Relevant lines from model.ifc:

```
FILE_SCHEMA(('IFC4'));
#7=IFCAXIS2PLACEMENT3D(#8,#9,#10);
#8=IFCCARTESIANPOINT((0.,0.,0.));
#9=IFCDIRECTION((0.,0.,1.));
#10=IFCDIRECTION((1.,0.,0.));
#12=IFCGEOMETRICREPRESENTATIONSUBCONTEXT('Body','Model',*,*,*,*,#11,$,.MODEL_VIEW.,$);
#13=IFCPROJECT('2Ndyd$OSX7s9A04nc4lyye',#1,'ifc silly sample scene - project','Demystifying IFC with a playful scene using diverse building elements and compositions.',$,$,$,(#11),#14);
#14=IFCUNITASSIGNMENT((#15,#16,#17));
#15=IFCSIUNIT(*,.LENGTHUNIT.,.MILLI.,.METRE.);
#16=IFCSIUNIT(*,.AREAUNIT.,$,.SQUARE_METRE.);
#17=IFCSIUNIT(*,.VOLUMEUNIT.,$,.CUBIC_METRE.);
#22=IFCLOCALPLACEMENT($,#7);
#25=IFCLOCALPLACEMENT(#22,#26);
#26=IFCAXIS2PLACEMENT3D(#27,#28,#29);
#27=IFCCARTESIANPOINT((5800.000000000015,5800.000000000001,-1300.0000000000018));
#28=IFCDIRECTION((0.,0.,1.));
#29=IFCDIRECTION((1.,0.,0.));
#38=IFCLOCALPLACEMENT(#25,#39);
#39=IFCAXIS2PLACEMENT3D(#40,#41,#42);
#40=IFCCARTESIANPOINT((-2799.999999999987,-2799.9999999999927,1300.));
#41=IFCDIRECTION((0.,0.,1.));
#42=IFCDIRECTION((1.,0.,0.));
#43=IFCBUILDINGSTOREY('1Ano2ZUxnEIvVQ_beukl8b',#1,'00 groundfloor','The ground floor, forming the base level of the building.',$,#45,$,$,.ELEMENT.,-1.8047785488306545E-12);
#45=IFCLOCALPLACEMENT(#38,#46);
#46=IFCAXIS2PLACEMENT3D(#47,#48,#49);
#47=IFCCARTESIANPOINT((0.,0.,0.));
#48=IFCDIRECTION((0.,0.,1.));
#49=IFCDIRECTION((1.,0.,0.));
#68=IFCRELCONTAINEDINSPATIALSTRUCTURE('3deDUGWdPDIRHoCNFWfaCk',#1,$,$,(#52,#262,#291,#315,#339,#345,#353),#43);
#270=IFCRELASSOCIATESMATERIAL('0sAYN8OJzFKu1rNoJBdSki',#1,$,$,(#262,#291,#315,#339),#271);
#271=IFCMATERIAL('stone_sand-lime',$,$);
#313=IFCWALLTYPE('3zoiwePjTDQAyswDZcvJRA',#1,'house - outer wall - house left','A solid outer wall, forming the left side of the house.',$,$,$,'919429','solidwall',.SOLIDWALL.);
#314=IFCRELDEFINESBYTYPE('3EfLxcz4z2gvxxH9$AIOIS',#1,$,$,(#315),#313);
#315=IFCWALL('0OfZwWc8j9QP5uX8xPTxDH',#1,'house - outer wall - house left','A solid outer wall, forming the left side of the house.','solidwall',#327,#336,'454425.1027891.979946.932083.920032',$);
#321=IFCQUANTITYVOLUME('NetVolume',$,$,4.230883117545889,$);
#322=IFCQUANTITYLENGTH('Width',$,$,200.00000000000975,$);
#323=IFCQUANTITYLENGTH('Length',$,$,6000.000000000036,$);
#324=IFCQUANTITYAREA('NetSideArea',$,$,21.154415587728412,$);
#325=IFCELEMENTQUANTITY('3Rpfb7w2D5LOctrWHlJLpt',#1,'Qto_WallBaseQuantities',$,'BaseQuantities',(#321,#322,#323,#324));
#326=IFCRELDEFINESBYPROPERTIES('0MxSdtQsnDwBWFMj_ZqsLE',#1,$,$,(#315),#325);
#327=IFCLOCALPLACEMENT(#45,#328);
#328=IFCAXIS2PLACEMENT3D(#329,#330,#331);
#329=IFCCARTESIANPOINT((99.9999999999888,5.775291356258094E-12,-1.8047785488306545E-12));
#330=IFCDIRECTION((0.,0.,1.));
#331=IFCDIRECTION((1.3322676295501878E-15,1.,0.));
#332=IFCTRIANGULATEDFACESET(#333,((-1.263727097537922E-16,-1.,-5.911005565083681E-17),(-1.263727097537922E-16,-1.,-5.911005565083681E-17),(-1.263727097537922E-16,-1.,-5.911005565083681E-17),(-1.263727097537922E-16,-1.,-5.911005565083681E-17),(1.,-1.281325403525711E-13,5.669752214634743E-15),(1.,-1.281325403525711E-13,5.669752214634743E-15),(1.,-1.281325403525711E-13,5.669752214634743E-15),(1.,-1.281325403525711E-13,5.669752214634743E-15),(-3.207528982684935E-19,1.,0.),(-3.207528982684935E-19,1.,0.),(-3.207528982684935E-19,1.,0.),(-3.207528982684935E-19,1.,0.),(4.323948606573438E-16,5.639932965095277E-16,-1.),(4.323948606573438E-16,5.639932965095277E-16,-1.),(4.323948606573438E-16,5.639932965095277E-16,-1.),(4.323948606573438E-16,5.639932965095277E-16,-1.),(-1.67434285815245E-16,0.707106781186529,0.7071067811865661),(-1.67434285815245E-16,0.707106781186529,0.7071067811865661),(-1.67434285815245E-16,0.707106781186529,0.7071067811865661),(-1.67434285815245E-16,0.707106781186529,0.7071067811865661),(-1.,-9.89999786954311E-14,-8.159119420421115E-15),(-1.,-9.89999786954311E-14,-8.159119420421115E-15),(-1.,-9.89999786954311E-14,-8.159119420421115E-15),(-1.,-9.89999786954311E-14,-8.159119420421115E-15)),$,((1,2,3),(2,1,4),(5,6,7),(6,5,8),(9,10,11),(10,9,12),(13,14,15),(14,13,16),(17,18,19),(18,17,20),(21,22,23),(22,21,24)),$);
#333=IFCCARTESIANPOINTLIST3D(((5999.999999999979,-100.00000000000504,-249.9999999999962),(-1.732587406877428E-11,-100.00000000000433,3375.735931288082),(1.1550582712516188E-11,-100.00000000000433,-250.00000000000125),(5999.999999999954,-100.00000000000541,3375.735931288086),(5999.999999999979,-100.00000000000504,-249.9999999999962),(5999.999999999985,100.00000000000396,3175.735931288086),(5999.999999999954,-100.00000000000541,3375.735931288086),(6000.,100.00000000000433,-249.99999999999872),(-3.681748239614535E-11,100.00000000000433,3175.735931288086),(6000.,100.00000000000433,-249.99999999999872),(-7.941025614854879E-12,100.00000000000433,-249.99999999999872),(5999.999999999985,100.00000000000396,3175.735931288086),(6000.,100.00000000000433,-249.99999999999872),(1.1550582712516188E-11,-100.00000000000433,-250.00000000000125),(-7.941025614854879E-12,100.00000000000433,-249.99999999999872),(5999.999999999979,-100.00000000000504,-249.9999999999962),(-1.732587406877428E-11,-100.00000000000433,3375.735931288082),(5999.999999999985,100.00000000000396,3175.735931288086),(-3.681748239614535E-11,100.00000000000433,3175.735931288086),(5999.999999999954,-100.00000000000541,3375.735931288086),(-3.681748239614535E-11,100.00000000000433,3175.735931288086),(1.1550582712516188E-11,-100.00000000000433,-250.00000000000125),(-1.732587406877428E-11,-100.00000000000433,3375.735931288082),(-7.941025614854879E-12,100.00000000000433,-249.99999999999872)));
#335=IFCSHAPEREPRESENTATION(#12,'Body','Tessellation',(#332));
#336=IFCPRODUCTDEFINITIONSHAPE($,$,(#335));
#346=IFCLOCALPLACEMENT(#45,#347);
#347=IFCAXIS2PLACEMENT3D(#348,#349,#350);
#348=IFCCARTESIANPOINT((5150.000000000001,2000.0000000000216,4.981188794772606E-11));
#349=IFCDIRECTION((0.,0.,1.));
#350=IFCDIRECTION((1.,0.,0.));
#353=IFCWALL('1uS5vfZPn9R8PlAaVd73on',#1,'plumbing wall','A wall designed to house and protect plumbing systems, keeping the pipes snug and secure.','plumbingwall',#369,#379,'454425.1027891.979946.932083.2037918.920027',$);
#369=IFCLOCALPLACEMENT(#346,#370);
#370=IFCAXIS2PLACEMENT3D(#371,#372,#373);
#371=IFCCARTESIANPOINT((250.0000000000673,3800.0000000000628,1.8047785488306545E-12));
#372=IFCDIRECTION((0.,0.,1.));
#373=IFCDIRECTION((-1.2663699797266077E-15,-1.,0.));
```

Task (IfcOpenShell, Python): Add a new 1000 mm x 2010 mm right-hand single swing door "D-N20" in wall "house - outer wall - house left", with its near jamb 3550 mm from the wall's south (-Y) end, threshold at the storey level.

```python
import numpy as np
import ifcopenshell
import ifcopenshell.api.feature
import ifcopenshell.api.geometry
import ifcopenshell.api.pset
import ifcopenshell.api.root
import ifcopenshell.api.spatial
import ifcopenshell.geom
import ifcopenshell.util.element
import ifcopenshell.util.placement
import ifcopenshell.util.representation
import ifcopenshell.util.shape
import ifcopenshell.util.unit

model = ifcopenshell.open("model.ifc")
unit_scale = ifcopenshell.util.unit.calculate_unit_scale(model)
area_scale = ifcopenshell.util.unit.calculate_unit_scale(model, "AREAUNIT")
volume_scale = ifcopenshell.util.unit.calculate_unit_scale(model, "VOLUMEUNIT")
settings = ifcopenshell.geom.settings()


def volume(element):
    """Net volume in cubic metres, openings subtracted."""
    shape = ifcopenshell.geom.create_shape(settings, element)
    return ifcopenshell.util.shape.get_volume(shape.geometry)


wall = model.by_guid("0OfZwWc8j9QP5uX8xPTxDH")
storey = ifcopenshell.util.element.get_container(wall, ifc_class="IfcBuildingStorey")
context = ifcopenshell.util.representation.get_context(model, "Model", "Body", "MODEL_VIEW")
before = volume(wall)

width, height, from_end, sill = 1, 2.01, 3.55, 0.0  # metres

# The wall runs along its own X axis, and the end named is its -X end.
wall_shape = ifcopenshell.geom.create_shape(settings, wall)
x, y, z = ifcopenshell.util.shape.get_vertices(wall_shape.geometry).T
start = x.min() + from_end
face, thickness = float(y.min()), float(y.max() - y.min())
wall_matrix = ifcopenshell.util.placement.get_local_placement(wall.ObjectPlacement)
level = ifcopenshell.util.placement.get_local_placement(storey.ObjectPlacement)[2, 3]


def in_wall(x, y):
    """Placement at x, y metres in the wall's axes, at sill height."""
    matrix = wall_matrix.copy()
    matrix[:, 3] = wall_matrix @ np.array([x / unit_scale, y / unit_scale, 0.0, 1.0])
    matrix[2, 3] = level + sill / unit_scale
    return matrix


# Opening: a box that overshoots both wall faces by 50 mm.
opening = ifcopenshell.api.root.create_entity(model, ifc_class="IfcOpeningElement", predefined_type="OPENING")
box = ifcopenshell.api.geometry.add_wall_representation(
    model, context=context, length=width, height=height, thickness=thickness + 0.1
)
ifcopenshell.api.geometry.assign_representation(model, product=opening, representation=box)
ifcopenshell.api.geometry.edit_object_placement(model, product=opening, matrix=in_wall(start, face - 0.05), is_si=False)
ifcopenshell.api.feature.add_feature(model, feature=opening, element=wall)

door = ifcopenshell.api.root.create_entity(model, ifc_class="IfcDoor", name="D-N20", predefined_type="DOOR")
door.OverallWidth, door.OverallHeight = width / unit_scale, height / unit_scale
door.OperationType = "SINGLE_SWING_RIGHT"
body = ifcopenshell.api.geometry.add_door_representation(
    model,
    context=context,
    overall_width=door.OverallWidth,
    overall_height=door.OverallHeight,
    operation_type="SINGLE_SWING_RIGHT",
    lining_properties={"LiningDepth": thickness / unit_scale, "ThresholdDepth": thickness / unit_scale},
)
ifcopenshell.api.geometry.assign_representation(model, product=door, representation=body)
ifcopenshell.api.spatial.assign_container(model, products=[door], relating_structure=storey)
ifcopenshell.api.feature.add_filling(model, opening=opening, element=door)

# The lining spans the wall, so the door starts at the wall face.
ifcopenshell.api.geometry.edit_object_placement(model, product=door, matrix=in_wall(start, face), is_si=False)

after = volume(wall)

# Update the wall's stored quantities.
qto = model.by_id(ifcopenshell.util.element.get_pset(wall, "Qto_WallBaseQuantities", should_inherit=False)["id"])
ifcopenshell.api.pset.edit_qto(model, qto=qto, properties={
    "NetVolume": after / volume_scale,
    "NetSideArea": after / thickness / area_scale,
})

print(f"wall volume {before:.3f} -> {after:.3f} m3")

model.write("model_edited.ifc")
```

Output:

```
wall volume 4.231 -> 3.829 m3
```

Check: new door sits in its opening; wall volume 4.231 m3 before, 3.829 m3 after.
